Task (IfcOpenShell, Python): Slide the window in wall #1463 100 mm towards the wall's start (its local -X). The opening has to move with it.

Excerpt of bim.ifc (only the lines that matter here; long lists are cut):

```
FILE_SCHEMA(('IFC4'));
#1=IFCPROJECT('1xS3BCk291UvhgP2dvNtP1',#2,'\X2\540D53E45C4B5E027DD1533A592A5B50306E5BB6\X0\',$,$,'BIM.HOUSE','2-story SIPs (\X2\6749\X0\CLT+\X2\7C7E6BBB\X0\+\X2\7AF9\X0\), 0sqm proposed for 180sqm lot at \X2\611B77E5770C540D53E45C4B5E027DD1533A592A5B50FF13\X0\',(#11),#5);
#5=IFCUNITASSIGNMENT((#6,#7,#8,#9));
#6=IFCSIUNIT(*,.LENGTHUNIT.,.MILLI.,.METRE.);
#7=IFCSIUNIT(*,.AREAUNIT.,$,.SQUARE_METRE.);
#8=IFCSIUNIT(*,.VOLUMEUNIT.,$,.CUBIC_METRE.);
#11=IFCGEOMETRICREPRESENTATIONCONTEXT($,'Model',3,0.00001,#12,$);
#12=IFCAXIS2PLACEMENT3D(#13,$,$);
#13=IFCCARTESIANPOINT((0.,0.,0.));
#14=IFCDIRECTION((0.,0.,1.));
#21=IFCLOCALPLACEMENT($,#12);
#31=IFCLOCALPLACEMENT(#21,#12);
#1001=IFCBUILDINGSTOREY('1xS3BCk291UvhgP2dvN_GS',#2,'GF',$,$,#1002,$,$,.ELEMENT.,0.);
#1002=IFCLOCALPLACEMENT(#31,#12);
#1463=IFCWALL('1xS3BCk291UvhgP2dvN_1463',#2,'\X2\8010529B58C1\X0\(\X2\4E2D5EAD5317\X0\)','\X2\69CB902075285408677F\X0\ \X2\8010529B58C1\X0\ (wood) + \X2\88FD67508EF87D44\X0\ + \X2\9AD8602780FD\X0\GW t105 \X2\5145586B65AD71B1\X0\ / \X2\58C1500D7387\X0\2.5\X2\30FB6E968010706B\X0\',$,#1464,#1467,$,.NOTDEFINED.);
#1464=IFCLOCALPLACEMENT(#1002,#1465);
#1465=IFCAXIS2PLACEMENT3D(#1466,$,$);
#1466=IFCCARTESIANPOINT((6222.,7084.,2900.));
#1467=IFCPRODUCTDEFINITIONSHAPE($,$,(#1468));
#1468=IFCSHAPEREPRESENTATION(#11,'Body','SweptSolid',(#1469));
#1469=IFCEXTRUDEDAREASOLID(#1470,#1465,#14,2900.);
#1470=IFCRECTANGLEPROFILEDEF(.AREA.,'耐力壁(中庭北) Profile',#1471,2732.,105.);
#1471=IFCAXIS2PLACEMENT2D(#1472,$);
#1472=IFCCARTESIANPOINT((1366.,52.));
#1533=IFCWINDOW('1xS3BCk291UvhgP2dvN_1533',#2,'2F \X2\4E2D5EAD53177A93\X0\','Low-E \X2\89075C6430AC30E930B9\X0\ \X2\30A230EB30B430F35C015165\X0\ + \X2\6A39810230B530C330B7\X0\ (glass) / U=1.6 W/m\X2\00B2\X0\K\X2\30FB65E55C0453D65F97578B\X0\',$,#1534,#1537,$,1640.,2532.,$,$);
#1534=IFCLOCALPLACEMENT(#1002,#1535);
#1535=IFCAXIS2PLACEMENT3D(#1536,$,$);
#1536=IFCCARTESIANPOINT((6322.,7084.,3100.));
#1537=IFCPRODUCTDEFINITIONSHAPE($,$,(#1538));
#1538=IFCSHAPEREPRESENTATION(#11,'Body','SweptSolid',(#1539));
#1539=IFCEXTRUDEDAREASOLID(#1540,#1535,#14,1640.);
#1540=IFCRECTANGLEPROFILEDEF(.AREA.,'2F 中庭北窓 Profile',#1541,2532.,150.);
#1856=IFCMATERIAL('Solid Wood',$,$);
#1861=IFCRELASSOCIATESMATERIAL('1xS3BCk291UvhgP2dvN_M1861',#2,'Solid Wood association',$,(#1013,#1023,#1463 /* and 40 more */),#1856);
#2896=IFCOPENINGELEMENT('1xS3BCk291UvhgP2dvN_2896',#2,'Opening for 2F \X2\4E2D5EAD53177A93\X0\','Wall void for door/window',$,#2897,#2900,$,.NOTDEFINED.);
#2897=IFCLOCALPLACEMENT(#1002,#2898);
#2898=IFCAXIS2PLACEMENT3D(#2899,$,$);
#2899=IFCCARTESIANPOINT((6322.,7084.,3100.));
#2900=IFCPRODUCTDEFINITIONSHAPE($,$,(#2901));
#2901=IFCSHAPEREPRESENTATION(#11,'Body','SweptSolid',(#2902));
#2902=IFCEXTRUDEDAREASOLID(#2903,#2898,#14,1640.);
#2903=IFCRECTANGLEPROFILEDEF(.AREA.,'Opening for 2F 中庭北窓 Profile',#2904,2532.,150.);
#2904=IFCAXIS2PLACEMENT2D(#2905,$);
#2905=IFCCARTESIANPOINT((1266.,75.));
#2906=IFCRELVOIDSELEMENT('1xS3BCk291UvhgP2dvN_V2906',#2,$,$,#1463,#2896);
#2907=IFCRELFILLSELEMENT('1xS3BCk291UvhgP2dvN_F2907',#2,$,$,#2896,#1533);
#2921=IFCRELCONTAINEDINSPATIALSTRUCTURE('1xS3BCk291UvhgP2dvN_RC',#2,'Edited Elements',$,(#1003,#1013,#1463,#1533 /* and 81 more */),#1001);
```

```python
import ifcopenshell
import ifcopenshell.api.geometry
import ifcopenshell.util.placement

model = ifcopenshell.open("bim.ifc")

window = model.by_guid("1xS3BCk291UvhgP2dvN_1533")
opening = window.FillsVoids[0].RelatingOpeningElement
wall = opening.VoidsElements[0].RelatingBuildingElement

wall_matrix = ifcopenshell.util.placement.get_local_placement(wall.ObjectPlacement)
shift = wall_matrix[:3, 0] * -100.0
before = ifcopenshell.util.placement.get_local_placement(window.ObjectPlacement)[:3, 3].copy()

# The window is not placed relative to its opening, so move both.
for product in (opening, window):
    matrix = ifcopenshell.util.placement.get_local_placement(product.ObjectPlacement)
    matrix[:3, 3] += shift
    ifcopenshell.api.geometry.edit_object_placement(model, product=product, matrix=matrix, is_si=False)

after = ifcopenshell.util.placement.get_local_placement(window.ObjectPlacement)[:3, 3]
print("window moved by", (after - before).round(3) + 0.0)

model.write("bim-out.ifc")
```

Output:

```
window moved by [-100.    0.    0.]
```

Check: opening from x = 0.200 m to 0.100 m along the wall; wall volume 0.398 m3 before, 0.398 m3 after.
